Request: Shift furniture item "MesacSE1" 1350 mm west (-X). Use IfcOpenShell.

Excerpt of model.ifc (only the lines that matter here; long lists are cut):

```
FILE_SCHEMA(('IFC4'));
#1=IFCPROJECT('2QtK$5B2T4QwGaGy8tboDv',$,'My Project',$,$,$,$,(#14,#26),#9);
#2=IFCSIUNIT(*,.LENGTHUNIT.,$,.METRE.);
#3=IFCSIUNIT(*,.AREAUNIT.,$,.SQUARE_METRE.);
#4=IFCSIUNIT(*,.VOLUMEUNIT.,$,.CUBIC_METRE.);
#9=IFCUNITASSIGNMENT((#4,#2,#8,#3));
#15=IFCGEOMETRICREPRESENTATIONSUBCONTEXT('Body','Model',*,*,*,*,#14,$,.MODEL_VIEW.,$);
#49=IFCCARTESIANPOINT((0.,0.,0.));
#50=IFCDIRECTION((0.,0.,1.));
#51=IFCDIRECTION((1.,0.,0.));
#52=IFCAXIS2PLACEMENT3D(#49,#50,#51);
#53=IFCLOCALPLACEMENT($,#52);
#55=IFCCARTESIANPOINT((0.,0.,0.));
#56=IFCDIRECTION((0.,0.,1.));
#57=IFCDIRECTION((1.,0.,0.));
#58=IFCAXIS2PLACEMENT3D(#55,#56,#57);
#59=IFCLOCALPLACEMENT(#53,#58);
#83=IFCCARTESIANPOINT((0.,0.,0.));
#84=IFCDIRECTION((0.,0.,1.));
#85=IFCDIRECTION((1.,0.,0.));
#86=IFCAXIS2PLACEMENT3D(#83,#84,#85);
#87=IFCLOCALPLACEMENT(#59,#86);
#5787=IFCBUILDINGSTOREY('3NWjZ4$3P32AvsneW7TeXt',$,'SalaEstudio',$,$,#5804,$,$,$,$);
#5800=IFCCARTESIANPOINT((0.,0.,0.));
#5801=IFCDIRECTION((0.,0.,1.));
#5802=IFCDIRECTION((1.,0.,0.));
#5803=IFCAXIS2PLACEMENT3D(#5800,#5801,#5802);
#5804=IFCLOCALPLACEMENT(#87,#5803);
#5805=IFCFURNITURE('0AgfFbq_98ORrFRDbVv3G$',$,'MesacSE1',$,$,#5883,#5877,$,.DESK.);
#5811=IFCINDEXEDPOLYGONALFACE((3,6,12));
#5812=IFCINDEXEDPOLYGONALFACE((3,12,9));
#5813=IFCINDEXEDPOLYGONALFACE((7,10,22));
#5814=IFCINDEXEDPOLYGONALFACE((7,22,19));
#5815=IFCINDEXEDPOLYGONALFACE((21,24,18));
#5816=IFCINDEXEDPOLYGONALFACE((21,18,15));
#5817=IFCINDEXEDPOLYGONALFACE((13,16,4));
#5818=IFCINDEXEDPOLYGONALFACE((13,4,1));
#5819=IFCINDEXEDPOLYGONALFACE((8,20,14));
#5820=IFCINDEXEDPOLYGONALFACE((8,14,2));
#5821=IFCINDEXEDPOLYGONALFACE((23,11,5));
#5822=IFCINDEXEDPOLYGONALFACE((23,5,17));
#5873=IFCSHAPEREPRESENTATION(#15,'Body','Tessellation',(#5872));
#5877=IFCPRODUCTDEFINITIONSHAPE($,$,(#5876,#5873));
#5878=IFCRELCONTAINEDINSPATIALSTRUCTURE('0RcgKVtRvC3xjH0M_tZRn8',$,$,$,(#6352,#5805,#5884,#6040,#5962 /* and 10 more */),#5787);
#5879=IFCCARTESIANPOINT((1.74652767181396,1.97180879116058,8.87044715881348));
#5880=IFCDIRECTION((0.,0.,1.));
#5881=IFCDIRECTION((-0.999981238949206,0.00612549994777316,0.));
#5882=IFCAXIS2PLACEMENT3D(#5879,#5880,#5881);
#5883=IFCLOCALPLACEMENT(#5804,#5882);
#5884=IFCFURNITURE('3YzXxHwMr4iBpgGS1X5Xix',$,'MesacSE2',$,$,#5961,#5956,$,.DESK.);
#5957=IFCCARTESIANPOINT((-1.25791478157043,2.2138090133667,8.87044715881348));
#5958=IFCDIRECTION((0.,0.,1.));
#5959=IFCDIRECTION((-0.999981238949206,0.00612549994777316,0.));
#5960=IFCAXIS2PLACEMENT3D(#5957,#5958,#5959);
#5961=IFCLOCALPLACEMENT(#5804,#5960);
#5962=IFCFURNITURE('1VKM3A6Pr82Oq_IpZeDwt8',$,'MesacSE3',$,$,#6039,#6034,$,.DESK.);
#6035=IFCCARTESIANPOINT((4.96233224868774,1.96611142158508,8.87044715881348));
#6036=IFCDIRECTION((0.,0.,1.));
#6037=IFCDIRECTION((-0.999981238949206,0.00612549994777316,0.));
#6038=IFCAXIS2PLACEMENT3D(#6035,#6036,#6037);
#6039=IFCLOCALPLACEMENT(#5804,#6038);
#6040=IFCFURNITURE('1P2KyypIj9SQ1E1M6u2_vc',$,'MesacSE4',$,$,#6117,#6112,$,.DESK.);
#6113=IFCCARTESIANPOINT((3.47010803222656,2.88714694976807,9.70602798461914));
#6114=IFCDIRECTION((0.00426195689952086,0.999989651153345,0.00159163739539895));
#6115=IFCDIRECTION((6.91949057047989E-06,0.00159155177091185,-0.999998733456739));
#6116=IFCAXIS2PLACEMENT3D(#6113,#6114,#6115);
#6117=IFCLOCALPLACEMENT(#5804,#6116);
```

```python
import ifcopenshell
import ifcopenshell.api.geometry
import ifcopenshell.util.placement

model = ifcopenshell.open("model.ifc")

item = model.by_id(5805)
matrix = ifcopenshell.util.placement.get_local_placement(item.ObjectPlacement)
matrix[0, 3] -= 1.35
ifcopenshell.api.geometry.edit_object_placement(model, product=item, matrix=matrix, is_si=False)

print(ifcopenshell.util.placement.get_local_placement(item.ObjectPlacement).round(3) + 0.0)

model.write("model_v2.ifc")
```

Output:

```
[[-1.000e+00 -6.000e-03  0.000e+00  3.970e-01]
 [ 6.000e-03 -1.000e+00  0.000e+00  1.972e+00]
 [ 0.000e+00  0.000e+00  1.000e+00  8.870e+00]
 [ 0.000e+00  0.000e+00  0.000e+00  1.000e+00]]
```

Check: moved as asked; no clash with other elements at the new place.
